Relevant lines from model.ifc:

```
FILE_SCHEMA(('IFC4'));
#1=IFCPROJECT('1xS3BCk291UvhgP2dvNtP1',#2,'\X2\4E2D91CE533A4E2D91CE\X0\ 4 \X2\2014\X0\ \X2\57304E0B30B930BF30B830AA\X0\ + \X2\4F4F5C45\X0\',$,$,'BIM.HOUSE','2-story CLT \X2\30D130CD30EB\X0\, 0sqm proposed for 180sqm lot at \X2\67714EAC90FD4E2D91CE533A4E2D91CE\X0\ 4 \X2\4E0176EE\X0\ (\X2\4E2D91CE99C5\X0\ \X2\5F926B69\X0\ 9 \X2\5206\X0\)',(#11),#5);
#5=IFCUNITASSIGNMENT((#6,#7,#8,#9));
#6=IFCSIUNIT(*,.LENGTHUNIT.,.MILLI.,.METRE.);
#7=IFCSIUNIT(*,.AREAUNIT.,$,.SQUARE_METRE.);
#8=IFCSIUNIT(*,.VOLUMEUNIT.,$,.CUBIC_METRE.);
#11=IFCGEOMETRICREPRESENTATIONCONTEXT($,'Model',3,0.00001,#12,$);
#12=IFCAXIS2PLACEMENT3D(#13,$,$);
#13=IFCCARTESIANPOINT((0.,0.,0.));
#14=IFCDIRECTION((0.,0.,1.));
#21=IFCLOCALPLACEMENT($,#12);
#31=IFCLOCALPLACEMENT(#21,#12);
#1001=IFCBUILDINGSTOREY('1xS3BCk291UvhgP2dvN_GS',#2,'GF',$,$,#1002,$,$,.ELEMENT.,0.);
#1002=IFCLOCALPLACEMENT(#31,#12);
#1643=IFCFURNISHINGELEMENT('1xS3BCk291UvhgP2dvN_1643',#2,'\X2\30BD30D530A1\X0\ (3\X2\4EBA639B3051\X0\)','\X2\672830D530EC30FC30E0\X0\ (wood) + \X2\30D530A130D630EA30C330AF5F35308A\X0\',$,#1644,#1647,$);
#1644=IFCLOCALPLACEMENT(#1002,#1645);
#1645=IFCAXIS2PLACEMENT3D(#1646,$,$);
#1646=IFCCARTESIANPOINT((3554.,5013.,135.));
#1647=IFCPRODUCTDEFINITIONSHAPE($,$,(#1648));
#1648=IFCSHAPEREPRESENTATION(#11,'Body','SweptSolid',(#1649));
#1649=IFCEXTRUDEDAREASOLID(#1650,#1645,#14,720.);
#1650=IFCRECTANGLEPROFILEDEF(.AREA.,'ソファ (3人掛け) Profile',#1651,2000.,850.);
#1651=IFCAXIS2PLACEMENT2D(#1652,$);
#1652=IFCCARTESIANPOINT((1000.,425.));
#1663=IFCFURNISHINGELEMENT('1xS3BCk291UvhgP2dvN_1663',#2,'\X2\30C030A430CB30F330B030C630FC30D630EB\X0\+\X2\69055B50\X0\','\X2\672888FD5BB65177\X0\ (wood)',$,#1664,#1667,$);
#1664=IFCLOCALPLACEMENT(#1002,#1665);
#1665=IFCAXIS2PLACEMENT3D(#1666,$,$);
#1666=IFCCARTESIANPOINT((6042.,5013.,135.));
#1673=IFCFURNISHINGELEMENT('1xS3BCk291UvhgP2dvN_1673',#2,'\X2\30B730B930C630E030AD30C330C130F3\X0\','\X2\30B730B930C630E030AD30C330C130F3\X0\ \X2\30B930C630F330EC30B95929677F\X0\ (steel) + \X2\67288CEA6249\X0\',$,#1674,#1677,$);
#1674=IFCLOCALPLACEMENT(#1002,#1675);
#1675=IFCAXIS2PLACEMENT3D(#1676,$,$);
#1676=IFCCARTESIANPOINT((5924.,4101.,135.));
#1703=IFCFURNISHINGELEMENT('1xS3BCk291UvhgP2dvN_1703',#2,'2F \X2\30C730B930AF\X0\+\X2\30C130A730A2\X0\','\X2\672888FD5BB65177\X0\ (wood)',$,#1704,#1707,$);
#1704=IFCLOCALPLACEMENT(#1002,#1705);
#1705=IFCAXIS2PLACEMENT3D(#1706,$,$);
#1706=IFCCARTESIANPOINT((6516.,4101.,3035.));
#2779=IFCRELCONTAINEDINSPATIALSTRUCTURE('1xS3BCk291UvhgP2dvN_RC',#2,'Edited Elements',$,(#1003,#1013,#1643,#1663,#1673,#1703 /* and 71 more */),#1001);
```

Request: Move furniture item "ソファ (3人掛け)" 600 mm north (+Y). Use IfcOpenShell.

```python
import ifcopenshell
import ifcopenshell.api.geometry
import ifcopenshell.util.placement
import ifcopenshell.util.unit

model = ifcopenshell.open("model.ifc")
unit_scale = ifcopenshell.util.unit.calculate_unit_scale(model)

item = model.by_id(1643)
matrix = ifcopenshell.util.placement.get_local_placement(item.ObjectPlacement)
matrix[1, 3] += 0.6 / unit_scale
ifcopenshell.api.geometry.edit_object_placement(model, product=item, matrix=matrix, is_si=False)

print(ifcopenshell.util.placement.get_local_placement(item.ObjectPlacement).round(3) + 0.0)

model.write("model-out.ifc")
```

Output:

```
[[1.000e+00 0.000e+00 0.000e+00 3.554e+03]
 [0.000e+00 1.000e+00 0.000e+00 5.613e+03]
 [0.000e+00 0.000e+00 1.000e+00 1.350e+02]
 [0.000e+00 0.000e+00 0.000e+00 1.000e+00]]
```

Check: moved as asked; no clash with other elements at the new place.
